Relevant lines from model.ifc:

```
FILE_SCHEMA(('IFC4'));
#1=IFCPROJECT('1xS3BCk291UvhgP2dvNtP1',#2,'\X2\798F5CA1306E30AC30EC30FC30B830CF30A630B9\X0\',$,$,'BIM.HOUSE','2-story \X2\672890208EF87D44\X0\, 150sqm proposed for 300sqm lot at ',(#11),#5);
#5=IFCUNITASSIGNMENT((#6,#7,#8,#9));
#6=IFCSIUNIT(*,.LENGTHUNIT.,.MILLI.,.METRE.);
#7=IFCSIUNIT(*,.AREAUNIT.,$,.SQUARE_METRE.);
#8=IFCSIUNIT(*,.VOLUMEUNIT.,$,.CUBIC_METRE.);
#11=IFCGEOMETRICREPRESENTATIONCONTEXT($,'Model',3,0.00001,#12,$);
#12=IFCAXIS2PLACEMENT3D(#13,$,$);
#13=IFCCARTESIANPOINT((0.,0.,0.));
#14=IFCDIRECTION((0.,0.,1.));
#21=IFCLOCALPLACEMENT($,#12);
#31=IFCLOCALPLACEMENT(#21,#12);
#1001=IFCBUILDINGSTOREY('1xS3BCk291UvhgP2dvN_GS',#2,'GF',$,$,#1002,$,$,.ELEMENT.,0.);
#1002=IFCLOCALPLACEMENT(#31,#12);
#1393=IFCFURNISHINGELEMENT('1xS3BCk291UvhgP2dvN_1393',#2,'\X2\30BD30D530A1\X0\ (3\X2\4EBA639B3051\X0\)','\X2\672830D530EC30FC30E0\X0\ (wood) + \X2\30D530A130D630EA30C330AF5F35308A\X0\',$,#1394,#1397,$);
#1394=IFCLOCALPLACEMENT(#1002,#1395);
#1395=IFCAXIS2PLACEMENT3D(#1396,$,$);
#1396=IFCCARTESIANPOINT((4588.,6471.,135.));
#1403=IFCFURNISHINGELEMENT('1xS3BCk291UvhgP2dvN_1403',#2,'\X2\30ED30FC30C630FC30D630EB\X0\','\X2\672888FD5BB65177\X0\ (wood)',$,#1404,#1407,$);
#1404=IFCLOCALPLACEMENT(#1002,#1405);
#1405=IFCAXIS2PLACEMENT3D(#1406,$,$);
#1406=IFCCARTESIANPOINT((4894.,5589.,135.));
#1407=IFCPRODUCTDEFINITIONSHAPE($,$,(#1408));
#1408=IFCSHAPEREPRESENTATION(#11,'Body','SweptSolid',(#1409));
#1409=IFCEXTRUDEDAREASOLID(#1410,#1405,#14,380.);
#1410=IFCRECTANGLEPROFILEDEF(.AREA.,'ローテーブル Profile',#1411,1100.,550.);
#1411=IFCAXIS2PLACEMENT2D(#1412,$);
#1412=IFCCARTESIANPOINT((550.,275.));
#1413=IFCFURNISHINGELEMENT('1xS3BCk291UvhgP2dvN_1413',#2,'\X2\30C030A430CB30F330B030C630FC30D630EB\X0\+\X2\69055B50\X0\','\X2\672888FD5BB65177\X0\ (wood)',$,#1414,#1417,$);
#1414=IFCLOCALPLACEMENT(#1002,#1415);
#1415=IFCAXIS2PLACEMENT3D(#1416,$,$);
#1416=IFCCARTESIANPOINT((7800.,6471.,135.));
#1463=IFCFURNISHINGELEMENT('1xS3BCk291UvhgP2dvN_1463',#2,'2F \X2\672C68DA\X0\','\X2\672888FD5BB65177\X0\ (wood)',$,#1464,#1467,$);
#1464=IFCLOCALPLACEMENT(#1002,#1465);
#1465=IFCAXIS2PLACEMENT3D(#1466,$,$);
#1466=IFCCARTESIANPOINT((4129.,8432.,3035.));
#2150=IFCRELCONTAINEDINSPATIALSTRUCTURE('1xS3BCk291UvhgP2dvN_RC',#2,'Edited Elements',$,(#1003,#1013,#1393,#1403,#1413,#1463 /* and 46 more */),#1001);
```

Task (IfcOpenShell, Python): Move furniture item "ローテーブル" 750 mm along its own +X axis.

```python
import ifcopenshell
import ifcopenshell.api.geometry
import ifcopenshell.util.placement

model = ifcopenshell.open("model.ifc")

item = model.by_guid("1xS3BCk291UvhgP2dvN_1403")
matrix = ifcopenshell.util.placement.get_local_placement(item.ObjectPlacement)
matrix[:3, 3] += matrix[:3, 0] * 750.0
ifcopenshell.api.geometry.edit_object_placement(model, product=item, matrix=matrix, is_si=False)

print(ifcopenshell.util.placement.get_local_placement(item.ObjectPlacement).round(3) + 0.0)

model.write("model_v2.ifc")
```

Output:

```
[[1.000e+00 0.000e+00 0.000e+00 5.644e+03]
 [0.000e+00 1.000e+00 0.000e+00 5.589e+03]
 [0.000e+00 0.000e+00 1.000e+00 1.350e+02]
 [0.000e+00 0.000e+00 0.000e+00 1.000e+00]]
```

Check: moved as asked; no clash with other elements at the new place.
